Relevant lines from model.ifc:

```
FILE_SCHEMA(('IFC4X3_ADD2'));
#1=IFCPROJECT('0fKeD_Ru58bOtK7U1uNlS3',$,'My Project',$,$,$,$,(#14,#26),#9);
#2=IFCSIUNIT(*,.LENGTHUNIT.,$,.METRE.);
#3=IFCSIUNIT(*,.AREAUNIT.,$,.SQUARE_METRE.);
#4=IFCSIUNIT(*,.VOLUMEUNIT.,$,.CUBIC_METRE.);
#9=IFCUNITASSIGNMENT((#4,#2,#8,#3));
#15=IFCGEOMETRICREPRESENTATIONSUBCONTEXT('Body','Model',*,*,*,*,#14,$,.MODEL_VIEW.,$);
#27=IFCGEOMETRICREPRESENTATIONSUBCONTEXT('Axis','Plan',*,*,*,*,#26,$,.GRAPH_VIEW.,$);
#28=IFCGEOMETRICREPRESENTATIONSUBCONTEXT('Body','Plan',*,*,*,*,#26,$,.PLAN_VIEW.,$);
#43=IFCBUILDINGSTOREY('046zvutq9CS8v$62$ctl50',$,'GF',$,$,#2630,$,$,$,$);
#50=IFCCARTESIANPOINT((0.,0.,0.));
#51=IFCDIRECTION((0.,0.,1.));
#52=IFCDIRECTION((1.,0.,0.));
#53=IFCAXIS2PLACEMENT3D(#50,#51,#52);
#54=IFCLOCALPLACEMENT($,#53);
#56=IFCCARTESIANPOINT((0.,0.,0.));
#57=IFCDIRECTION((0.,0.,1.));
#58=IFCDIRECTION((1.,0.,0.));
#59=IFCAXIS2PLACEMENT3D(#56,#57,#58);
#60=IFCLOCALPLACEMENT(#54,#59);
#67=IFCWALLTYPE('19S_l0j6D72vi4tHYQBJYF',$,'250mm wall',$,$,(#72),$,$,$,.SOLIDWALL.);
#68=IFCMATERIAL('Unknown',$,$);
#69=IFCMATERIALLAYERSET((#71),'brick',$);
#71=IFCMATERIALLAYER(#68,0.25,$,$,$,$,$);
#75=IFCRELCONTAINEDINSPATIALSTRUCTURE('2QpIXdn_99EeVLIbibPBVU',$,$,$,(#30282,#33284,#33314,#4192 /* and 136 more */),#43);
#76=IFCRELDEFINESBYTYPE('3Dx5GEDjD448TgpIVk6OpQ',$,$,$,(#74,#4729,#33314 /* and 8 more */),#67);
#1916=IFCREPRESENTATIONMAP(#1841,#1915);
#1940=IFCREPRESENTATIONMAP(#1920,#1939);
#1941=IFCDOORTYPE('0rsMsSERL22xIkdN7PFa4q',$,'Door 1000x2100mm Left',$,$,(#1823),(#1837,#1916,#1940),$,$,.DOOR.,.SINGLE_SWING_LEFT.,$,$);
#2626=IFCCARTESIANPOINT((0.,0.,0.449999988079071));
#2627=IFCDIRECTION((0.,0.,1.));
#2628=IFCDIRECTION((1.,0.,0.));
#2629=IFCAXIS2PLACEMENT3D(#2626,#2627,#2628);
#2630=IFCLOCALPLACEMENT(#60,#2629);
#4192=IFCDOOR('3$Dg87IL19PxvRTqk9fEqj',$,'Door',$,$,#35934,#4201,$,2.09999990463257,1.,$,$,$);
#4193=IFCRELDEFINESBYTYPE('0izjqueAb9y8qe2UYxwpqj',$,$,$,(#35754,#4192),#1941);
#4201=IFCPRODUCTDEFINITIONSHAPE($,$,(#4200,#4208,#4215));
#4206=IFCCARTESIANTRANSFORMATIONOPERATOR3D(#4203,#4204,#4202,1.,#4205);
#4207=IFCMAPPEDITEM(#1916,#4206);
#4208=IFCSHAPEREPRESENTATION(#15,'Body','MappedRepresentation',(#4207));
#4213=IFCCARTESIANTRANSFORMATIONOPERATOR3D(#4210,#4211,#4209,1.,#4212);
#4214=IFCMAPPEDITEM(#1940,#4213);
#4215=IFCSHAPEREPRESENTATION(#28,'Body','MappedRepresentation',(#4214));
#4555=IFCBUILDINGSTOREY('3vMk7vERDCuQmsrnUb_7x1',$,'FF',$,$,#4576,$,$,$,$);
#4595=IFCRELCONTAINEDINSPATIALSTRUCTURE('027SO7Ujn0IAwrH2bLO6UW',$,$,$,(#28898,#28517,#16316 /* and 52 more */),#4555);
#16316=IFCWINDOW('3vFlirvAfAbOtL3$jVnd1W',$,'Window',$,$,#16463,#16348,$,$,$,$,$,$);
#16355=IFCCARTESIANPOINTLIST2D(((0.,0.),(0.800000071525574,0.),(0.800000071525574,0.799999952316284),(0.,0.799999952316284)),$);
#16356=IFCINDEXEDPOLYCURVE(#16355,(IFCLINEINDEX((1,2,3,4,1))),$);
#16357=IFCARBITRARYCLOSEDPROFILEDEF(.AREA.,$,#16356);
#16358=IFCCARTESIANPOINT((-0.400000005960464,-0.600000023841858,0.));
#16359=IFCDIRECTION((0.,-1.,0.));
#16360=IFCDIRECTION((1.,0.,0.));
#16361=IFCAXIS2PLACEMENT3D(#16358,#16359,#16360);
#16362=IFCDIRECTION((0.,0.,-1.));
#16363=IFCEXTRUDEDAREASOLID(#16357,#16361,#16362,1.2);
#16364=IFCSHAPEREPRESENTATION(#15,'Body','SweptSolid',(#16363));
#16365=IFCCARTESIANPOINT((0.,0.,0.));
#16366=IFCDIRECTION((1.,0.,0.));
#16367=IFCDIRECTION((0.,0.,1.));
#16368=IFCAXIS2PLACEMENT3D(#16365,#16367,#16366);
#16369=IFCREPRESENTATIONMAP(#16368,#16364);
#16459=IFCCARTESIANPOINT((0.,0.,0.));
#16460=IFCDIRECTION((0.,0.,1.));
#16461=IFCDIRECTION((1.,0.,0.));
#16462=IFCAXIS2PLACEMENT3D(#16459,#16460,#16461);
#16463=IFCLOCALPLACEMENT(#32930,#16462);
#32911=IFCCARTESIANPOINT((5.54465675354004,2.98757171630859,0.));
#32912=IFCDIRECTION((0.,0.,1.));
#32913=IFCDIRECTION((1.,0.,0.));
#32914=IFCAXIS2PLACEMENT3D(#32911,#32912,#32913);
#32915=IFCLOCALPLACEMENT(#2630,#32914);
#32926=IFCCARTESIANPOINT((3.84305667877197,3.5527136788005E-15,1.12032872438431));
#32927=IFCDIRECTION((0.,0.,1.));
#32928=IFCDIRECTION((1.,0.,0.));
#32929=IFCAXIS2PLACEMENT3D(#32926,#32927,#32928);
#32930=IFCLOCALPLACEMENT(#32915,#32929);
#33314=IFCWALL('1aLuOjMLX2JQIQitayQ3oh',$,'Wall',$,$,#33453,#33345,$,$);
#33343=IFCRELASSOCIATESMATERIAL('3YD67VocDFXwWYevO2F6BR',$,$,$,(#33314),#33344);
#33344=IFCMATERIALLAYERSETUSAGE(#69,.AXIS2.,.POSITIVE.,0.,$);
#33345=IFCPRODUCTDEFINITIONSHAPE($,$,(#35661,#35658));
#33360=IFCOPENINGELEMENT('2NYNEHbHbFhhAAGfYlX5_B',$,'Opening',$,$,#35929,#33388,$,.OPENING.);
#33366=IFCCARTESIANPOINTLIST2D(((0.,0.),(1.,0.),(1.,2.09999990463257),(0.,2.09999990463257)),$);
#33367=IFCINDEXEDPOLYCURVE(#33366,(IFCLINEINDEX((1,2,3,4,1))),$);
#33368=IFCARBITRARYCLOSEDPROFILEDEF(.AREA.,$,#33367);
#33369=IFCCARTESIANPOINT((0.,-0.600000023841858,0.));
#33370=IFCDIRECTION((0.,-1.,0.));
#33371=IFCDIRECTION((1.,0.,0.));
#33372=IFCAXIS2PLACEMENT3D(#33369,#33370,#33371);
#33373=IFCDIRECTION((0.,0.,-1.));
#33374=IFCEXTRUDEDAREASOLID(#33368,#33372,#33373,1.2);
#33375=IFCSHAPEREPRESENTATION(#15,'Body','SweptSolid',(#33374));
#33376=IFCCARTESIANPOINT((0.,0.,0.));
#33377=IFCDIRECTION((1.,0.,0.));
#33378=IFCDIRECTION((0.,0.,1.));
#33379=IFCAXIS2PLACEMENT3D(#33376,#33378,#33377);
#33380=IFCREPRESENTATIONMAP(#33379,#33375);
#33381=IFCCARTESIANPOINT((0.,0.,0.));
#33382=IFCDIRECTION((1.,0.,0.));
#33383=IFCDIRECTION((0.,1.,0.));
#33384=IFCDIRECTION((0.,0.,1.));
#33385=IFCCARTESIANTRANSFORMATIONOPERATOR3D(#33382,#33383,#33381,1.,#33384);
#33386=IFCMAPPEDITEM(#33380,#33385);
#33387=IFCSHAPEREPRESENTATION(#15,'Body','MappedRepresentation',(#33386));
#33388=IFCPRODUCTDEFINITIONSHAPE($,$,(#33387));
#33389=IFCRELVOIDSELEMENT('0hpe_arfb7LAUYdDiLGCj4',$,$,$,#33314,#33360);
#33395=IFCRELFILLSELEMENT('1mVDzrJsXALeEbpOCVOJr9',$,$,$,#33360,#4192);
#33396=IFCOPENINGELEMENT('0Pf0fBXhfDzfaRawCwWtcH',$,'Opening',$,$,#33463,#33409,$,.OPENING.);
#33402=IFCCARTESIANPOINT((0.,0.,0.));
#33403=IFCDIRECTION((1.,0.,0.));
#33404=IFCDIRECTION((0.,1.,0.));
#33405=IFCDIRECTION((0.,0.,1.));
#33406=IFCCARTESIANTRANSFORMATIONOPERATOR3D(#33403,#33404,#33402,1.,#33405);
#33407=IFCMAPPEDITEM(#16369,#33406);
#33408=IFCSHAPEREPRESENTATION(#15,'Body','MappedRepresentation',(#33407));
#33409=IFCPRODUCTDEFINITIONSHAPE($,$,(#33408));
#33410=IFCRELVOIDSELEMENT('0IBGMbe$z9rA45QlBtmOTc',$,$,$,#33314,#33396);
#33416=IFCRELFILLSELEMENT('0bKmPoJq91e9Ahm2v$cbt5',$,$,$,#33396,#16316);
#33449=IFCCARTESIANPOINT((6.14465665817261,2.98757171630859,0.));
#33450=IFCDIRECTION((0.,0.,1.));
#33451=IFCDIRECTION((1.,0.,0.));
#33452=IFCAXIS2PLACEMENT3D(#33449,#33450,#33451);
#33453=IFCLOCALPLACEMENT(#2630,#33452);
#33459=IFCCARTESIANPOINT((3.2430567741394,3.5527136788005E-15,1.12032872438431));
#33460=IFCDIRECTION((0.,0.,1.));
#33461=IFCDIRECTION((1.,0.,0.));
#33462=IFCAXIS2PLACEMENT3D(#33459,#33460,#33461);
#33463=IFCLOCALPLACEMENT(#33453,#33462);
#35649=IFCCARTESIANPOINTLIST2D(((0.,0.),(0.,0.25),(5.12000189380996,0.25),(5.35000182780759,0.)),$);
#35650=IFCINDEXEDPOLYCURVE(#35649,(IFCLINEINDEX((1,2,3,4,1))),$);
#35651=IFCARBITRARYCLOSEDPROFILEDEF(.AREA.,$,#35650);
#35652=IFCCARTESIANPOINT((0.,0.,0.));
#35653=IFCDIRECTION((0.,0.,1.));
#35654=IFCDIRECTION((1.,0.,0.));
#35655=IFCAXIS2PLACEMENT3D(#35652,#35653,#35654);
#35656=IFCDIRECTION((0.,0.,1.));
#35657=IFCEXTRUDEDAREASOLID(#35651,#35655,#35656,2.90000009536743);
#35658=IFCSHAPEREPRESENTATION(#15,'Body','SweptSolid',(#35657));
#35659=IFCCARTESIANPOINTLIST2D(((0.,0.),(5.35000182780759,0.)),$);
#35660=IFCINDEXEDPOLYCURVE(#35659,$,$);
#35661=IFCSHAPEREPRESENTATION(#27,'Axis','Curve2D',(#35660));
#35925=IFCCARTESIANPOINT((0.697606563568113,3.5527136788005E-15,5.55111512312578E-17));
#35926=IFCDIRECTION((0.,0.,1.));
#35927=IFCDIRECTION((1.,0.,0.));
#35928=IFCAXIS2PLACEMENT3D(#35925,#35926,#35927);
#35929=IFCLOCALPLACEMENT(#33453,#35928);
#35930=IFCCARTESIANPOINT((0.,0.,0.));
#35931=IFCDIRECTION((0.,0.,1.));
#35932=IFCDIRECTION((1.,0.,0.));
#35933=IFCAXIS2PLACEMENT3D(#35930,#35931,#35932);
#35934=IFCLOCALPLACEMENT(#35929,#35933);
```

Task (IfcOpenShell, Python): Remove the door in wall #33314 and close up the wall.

```python
import ifcopenshell
import ifcopenshell.api.feature
import ifcopenshell.api.root
import ifcopenshell.geom
import ifcopenshell.util.shape

model = ifcopenshell.open("model.ifc")
settings = ifcopenshell.geom.settings()


def volume(element):
    """Net volume in cubic metres, openings subtracted."""
    shape = ifcopenshell.geom.create_shape(settings, element)
    return ifcopenshell.util.shape.get_volume(shape.geometry)


door = model.by_guid("3$Dg87IL19PxvRTqk9fEqj")
opening = door.FillsVoids[0].RelatingOpeningElement
wall = opening.VoidsElements[0].RelatingBuildingElement
before = volume(wall)

ifcopenshell.api.root.remove_product(model, product=door)
ifcopenshell.api.feature.remove_feature(model, feature=opening)

after = volume(wall)

print(f"wall volume {before:.3f} -> {after:.3f} m3")

model.write("model_updated.ifc")
```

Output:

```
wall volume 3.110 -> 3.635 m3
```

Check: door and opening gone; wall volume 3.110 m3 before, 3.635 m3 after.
